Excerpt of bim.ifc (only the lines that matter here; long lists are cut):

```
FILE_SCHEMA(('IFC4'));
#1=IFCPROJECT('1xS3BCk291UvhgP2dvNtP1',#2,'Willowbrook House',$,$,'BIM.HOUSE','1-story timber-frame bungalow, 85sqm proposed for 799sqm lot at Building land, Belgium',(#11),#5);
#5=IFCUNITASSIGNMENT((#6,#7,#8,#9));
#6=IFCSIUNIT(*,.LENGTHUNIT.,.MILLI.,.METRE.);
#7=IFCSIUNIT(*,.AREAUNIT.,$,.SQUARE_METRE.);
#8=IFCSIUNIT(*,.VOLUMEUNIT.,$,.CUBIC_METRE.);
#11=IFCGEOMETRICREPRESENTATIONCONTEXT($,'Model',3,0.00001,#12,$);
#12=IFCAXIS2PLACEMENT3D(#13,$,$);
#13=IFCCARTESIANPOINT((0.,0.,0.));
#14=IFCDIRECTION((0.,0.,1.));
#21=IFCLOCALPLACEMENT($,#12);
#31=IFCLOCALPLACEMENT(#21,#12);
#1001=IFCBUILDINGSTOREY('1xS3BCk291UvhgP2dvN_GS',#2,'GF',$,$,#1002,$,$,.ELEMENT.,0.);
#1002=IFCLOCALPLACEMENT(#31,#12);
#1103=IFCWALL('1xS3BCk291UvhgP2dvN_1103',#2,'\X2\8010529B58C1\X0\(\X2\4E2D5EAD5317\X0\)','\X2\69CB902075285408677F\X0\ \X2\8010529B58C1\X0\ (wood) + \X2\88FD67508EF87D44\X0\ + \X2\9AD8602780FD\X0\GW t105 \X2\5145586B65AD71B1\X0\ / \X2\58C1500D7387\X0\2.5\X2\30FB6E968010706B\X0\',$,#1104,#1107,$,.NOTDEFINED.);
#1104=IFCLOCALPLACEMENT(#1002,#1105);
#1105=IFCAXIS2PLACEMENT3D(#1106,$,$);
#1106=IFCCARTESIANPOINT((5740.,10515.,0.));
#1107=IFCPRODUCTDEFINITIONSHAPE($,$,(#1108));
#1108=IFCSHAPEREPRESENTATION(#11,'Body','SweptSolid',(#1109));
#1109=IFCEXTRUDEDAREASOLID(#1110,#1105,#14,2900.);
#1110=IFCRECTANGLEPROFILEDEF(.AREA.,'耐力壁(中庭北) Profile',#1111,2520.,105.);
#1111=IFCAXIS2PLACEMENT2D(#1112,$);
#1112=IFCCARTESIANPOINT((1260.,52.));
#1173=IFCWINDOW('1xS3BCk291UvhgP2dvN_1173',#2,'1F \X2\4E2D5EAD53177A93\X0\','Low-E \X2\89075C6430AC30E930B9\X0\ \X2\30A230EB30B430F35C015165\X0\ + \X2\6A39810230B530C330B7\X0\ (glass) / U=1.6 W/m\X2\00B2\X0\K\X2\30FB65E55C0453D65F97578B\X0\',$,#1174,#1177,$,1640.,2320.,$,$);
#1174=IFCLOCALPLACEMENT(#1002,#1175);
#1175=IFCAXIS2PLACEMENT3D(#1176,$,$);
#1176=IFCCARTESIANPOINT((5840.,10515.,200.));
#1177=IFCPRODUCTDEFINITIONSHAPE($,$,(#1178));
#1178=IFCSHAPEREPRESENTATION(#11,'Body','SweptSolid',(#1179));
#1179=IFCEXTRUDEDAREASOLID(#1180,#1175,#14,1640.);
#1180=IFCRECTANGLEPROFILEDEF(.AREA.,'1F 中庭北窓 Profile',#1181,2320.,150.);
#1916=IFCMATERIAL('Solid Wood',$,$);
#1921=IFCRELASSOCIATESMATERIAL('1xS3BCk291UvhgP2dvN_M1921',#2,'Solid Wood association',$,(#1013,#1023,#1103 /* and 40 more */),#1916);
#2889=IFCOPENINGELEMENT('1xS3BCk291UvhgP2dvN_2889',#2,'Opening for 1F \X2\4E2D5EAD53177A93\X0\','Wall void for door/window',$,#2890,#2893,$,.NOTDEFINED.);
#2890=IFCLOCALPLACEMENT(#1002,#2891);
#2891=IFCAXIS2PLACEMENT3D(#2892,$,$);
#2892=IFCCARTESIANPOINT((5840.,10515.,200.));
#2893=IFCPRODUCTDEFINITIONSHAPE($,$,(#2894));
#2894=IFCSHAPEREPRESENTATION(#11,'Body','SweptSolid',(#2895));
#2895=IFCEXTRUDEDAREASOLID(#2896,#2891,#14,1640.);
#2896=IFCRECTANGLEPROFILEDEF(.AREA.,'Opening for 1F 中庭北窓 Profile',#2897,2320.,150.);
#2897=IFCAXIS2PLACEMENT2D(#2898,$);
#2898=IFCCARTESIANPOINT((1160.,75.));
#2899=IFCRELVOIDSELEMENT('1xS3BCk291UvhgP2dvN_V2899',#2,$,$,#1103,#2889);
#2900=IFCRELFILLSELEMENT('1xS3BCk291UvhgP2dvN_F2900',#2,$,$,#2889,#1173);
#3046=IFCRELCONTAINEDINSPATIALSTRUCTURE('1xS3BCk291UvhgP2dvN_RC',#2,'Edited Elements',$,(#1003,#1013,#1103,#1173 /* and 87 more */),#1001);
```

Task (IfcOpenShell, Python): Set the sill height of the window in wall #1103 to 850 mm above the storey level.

```python
import numpy as np
import ifcopenshell
import ifcopenshell.api.geometry
import ifcopenshell.geom
import ifcopenshell.util.element
import ifcopenshell.util.placement
import ifcopenshell.util.shape
import ifcopenshell.util.unit

model = ifcopenshell.open("bim.ifc")
unit_scale = ifcopenshell.util.unit.calculate_unit_scale(model)

window = model.by_id(1173)
opening = window.FillsVoids[0].RelatingOpeningElement
storey = ifcopenshell.util.element.get_container(window, ifc_class="IfcBuildingStorey")
level = ifcopenshell.util.placement.get_local_placement(storey.ObjectPlacement)[2, 3]

# The opening's origin need not be at the sill, so measure its lowest point.
shape = ifcopenshell.geom.create_shape(ifcopenshell.geom.settings(), opening)
bottom = ifcopenshell.util.shape.get_shape_bottom_elevation(shape, shape.geometry) / unit_scale
dz = level + 0.85 / unit_scale - bottom

shift = np.array([0.0, 0.0, dz])
# The window is not placed relative to its opening, so move both.
for product in (opening, window):
    matrix = ifcopenshell.util.placement.get_local_placement(product.ObjectPlacement)
    matrix[:3, 3] += shift
    ifcopenshell.api.geometry.edit_object_placement(model, product=product, matrix=matrix, is_si=False)

print(f"moved by {dz * unit_scale:+.3f} m")

model.write("bim_updated.ifc")
```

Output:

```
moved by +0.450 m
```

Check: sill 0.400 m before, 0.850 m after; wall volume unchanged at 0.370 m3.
